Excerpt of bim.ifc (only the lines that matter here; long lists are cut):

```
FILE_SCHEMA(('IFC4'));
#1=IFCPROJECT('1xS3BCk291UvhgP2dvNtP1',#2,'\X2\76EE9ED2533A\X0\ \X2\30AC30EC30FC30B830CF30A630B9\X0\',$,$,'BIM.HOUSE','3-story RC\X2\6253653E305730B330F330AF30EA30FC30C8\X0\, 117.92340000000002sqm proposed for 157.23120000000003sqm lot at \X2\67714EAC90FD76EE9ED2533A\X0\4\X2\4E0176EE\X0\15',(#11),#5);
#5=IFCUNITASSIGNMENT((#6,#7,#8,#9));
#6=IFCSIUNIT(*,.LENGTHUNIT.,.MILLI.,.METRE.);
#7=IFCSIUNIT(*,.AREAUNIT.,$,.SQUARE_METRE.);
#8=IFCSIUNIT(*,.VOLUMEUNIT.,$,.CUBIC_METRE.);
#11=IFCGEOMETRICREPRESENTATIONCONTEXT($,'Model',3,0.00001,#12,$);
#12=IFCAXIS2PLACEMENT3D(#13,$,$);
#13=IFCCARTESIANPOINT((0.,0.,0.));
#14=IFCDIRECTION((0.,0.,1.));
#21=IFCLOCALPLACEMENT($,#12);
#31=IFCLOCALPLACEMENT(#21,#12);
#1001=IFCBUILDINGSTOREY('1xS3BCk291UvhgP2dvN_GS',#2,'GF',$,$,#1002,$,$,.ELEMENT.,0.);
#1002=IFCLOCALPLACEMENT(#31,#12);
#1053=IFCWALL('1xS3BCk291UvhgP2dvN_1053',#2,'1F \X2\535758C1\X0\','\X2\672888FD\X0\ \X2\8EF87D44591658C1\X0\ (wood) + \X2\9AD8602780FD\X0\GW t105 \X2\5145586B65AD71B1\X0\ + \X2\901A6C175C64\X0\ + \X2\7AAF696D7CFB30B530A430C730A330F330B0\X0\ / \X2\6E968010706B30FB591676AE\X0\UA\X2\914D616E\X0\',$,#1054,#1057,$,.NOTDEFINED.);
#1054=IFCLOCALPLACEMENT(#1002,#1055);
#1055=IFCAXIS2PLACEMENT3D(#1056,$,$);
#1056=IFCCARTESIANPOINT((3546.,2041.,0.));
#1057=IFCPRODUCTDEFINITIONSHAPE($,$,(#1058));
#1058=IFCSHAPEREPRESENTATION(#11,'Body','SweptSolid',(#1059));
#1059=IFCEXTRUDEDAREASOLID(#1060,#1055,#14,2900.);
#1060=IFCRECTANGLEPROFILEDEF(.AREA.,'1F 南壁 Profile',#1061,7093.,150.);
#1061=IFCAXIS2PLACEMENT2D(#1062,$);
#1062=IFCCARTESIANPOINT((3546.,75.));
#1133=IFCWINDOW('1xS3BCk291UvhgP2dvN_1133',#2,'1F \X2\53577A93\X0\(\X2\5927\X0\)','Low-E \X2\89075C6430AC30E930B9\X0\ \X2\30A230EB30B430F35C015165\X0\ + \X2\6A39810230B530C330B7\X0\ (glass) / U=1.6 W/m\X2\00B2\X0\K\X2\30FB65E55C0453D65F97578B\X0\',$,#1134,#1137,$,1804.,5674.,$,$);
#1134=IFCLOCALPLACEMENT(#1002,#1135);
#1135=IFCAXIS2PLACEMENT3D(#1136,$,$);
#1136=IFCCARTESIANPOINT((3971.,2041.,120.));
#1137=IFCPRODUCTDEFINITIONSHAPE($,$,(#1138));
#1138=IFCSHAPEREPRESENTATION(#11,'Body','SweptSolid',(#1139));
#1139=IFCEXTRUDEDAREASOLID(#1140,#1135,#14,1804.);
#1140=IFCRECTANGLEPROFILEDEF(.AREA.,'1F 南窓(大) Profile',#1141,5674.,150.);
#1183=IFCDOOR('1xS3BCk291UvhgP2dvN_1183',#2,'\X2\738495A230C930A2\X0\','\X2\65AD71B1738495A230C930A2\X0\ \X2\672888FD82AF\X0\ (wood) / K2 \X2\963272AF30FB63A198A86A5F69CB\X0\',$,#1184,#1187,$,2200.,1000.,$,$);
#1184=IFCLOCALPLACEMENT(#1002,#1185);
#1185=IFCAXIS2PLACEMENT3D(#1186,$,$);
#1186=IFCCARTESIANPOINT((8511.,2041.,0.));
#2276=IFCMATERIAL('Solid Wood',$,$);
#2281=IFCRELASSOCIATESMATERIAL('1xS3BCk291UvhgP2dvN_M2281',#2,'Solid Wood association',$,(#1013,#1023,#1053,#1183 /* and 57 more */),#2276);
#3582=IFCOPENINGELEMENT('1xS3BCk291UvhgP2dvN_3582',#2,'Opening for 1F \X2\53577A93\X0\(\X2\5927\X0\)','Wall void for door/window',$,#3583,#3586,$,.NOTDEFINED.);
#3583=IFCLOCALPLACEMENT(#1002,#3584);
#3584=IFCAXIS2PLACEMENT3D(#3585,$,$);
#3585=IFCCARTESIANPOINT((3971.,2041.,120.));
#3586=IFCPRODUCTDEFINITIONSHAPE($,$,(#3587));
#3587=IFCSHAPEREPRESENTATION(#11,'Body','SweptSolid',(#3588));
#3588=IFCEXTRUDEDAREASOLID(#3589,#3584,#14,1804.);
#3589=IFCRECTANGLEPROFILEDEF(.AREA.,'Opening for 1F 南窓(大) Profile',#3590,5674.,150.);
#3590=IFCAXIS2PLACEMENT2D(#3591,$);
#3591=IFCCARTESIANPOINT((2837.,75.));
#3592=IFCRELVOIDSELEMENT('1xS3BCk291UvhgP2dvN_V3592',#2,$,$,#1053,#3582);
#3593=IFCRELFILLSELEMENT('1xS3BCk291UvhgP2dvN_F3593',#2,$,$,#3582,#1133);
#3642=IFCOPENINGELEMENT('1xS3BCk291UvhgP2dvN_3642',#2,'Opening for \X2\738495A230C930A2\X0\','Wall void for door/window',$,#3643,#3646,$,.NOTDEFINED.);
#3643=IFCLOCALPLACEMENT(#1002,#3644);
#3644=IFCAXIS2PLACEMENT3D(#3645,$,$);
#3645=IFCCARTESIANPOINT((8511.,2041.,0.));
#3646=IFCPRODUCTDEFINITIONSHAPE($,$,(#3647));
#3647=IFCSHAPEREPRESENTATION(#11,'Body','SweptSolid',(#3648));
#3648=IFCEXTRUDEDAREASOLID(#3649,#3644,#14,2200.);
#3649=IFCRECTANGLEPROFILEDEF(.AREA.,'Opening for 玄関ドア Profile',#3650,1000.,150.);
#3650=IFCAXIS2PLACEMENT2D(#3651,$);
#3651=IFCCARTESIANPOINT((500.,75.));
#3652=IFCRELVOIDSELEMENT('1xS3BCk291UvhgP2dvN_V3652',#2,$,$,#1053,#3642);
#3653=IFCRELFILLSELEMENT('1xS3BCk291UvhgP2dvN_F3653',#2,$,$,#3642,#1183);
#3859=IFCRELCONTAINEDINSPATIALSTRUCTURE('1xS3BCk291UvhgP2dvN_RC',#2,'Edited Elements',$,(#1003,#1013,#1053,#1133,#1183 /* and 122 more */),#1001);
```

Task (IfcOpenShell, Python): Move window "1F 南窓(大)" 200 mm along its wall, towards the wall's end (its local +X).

```python
import ifcopenshell
import ifcopenshell.api.geometry
import ifcopenshell.util.placement

model = ifcopenshell.open("bim.ifc")

window = model.by_guid("1xS3BCk291UvhgP2dvN_1133")
opening = window.FillsVoids[0].RelatingOpeningElement
wall = opening.VoidsElements[0].RelatingBuildingElement

wall_matrix = ifcopenshell.util.placement.get_local_placement(wall.ObjectPlacement)
shift = wall_matrix[:3, 0] * 200.0
before = ifcopenshell.util.placement.get_local_placement(window.ObjectPlacement)[:3, 3].copy()

# The window is not placed relative to its opening, so move both.
for product in (opening, window):
    matrix = ifcopenshell.util.placement.get_local_placement(product.ObjectPlacement)
    matrix[:3, 3] += shift
    ifcopenshell.api.geometry.edit_object_placement(model, product=product, matrix=matrix, is_si=False)

after = ifcopenshell.util.placement.get_local_placement(window.ObjectPlacement)[:3, 3]
print("window moved by", (after - before).round(3) + 0.0)

model.write("bim_edited.ifc")
```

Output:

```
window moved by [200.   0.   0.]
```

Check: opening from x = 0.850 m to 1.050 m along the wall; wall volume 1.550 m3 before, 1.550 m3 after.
